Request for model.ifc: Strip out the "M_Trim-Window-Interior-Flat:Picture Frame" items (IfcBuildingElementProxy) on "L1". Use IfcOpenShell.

First a look at what the model holds.

```python
import ifcopenshell
import ifcopenshell.util.element

model = ifcopenshell.open("model.ifc")
print(model.schema)
storey = next(s for s in model.by_type("IfcBuildingStorey") if s.Name == "L1")
proxies = [e for e in ifcopenshell.util.element.get_decomposition(storey) if e.is_a("IfcBuildingElementProxy")]
seen = {}
for e in proxies:
    element_type = ifcopenshell.util.element.get_type(e)
    name = element_type.Name if element_type not in (None, e) else None
    seen[name] = seen.get(name, 0) + 1
for name, count in sorted(seen.items(), key=str):
    print(count, "x", name)
```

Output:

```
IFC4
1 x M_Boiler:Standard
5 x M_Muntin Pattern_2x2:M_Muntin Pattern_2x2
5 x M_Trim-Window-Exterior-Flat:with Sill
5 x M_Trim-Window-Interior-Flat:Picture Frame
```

```python
import ifcopenshell
import ifcopenshell.api.root
import ifcopenshell.util.element

model = ifcopenshell.open("model.ifc")

storey = next(s for s in model.by_type("IfcBuildingStorey") if s.Name == "L1")
proxies = [e for e in ifcopenshell.util.element.get_decomposition(storey) if e.is_a("IfcBuildingElementProxy")]
targets = [e for e in proxies if (t := ifcopenshell.util.element.get_type(e)) not in (None, e) and t.Name == "M_Trim-Window-Interior-Flat:Picture Frame"]

for e in targets:
    ifcopenshell.api.root.remove_product(model, product=e)
print(len(targets), "removed")

model.write("model_rev.ifc")
```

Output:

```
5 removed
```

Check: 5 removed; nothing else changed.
